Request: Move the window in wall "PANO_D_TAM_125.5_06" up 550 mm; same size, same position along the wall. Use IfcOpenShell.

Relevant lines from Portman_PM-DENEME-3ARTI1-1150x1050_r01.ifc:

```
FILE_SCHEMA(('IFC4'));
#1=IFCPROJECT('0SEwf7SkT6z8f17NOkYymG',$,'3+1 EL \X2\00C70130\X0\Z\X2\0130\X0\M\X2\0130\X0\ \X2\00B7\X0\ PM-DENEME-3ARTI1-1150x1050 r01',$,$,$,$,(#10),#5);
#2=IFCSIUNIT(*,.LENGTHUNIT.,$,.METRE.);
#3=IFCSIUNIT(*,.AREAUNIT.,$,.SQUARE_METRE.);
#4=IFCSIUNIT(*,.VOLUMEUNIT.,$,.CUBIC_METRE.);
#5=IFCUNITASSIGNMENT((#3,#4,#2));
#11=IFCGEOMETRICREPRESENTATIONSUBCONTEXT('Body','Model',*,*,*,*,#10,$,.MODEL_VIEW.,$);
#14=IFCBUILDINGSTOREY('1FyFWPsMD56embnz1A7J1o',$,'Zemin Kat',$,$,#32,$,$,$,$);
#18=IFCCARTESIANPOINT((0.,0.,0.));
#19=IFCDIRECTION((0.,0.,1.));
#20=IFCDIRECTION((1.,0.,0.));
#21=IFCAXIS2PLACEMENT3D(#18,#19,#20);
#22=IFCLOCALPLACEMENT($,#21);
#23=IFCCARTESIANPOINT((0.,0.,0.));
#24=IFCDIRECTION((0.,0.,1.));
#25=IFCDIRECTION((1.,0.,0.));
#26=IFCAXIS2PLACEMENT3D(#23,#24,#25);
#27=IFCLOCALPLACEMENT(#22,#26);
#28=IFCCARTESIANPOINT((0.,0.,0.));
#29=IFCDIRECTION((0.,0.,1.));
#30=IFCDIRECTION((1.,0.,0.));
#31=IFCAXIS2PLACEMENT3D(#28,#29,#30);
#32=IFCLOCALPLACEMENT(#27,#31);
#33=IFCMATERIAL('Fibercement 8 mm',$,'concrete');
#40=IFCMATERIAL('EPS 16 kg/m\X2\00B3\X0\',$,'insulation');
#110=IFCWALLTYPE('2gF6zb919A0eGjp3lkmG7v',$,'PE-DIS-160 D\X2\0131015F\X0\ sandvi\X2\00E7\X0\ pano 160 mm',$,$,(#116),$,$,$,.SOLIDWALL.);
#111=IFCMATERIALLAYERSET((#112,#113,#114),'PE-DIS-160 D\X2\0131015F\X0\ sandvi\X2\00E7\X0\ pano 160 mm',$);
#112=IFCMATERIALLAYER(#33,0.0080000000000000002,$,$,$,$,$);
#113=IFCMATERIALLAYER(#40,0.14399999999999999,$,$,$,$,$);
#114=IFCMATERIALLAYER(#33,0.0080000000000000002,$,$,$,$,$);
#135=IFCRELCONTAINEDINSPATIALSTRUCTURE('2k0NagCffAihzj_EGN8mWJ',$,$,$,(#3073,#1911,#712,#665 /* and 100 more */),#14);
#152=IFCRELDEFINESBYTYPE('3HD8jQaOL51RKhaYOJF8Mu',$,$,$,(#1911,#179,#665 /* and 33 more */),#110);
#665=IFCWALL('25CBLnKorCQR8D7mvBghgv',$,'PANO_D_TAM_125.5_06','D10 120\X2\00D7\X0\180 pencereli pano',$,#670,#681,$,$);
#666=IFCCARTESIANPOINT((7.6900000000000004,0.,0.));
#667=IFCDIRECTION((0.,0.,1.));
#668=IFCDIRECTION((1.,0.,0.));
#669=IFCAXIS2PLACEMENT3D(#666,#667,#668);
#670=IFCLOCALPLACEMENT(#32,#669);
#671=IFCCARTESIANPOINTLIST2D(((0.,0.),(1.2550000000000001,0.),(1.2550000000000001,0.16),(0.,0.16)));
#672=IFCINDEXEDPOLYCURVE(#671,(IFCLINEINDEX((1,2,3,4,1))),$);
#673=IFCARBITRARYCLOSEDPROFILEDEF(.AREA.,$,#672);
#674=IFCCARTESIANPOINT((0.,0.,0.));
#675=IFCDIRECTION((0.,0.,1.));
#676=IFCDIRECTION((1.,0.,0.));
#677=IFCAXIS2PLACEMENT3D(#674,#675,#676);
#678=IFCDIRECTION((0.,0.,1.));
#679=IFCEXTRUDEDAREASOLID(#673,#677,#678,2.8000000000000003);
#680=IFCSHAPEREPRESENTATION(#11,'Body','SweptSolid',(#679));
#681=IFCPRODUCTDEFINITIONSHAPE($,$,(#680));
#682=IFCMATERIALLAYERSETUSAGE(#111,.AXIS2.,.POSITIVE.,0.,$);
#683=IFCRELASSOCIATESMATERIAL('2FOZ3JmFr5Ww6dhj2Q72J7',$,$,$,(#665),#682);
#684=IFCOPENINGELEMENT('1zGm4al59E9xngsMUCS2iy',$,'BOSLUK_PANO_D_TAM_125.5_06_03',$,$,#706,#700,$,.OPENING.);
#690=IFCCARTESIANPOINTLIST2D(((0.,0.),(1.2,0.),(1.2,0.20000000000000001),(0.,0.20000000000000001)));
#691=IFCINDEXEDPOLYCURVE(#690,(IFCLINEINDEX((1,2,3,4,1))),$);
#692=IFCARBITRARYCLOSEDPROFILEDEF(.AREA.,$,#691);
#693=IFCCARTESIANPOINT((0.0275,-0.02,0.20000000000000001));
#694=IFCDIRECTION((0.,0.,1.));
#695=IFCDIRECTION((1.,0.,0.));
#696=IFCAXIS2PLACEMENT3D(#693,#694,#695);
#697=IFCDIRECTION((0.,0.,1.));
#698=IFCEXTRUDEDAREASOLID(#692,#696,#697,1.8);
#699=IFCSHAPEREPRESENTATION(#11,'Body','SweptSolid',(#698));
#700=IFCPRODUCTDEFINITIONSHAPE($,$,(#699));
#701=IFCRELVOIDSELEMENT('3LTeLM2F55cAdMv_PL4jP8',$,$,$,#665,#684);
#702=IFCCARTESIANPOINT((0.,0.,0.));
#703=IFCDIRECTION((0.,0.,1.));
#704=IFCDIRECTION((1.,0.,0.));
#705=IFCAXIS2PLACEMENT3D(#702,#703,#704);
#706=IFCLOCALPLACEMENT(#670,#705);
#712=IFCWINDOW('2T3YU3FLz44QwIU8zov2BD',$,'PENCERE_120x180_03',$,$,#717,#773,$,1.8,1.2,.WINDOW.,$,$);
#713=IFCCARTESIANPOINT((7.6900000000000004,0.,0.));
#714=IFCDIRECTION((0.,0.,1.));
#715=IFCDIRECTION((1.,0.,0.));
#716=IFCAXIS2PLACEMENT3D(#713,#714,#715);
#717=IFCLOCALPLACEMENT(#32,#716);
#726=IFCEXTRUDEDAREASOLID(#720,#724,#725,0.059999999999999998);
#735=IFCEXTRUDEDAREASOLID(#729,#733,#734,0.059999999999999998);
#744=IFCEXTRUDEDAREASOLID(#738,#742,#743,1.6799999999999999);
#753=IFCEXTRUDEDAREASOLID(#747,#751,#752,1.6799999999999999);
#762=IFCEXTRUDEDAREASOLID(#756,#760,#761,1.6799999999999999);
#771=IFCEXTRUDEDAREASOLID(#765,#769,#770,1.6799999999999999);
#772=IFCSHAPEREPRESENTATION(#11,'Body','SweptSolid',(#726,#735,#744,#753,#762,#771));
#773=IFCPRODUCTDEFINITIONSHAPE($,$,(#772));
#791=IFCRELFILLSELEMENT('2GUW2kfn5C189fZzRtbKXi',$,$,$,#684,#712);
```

```python
import numpy as np
import ifcopenshell
import ifcopenshell.api.geometry
import ifcopenshell.util.placement
import ifcopenshell.util.unit

model = ifcopenshell.open("Portman_PM-DENEME-3ARTI1-1150x1050_r01.ifc")
unit_scale = ifcopenshell.util.unit.calculate_unit_scale(model)

window = model.by_id(712)
opening = window.FillsVoids[0].RelatingOpeningElement
dz = 0.55

shift = np.array([0.0, 0.0, dz])
# The window is not placed relative to its opening, so move both.
for product in (opening, window):
    matrix = ifcopenshell.util.placement.get_local_placement(product.ObjectPlacement)
    matrix[:3, 3] += shift
    ifcopenshell.api.geometry.edit_object_placement(model, product=product, matrix=matrix, is_si=False)

print(f"moved by {dz * unit_scale:+.3f} m")

model.write("Portman_PM-DENEME-3ARTI1-1150x1050_r01-out.ifc")
```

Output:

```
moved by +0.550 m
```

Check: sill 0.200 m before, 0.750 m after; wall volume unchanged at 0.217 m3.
